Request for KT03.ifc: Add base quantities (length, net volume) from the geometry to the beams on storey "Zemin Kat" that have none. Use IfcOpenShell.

First a look at what the model holds.

```python
import ifcopenshell
import ifcopenshell.util.element
import ifcopenshell.util.unit

model = ifcopenshell.open("KT03.ifc")
print(model.schema)
for unit_type in ("LENGTHUNIT", "AREAUNIT", "VOLUMEUNIT"):
    print(unit_type, ifcopenshell.util.unit.calculate_unit_scale(model, unit_type))
storey = next(s for s in model.by_type("IfcBuildingStorey") if s.Name == "Zemin Kat")
beams = [e for e in ifcopenshell.util.element.get_decomposition(storey) if e.is_a("IfcBeam")]
for e in sorted(beams, key=lambda e: e.id()):
    print(e.id(), e.is_a(), e.Name, list(ifcopenshell.util.element.get_psets(e, qtos_only=True)), sep=" | ")
```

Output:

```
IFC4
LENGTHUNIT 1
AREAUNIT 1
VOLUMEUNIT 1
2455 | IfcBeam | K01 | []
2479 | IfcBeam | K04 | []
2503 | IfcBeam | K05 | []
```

```python
import ifcopenshell
import ifcopenshell.api.pset
import ifcopenshell.geom
import ifcopenshell.util.element
import ifcopenshell.util.shape
import ifcopenshell.util.unit

model = ifcopenshell.open("KT03.ifc")
unit_scale = ifcopenshell.util.unit.calculate_unit_scale(model)
volume_scale = ifcopenshell.util.unit.calculate_unit_scale(model, "VOLUMEUNIT")
settings = ifcopenshell.geom.settings()

storey = next(s for s in model.by_type("IfcBuildingStorey") if s.Name == "Zemin Kat")
beams = [e for e in ifcopenshell.util.element.get_decomposition(storey) if e.is_a("IfcBeam")]

for e in sorted(beams, key=lambda e: e.id()):
    if ifcopenshell.util.element.get_psets(e, qtos_only=True, should_inherit=False):
        continue
    # Geometry comes back in metres, in the element's own axes.
    shape = ifcopenshell.geom.create_shape(settings, e)
    values = {
        "Length": ifcopenshell.util.shape.get_max_xyz(shape.geometry) / unit_scale,
        "NetVolume": ifcopenshell.util.shape.get_volume(shape.geometry) / volume_scale,
    }
    qto = ifcopenshell.api.pset.add_qto(model, product=e, name="Qto_BeamBaseQuantities")
    ifcopenshell.api.pset.edit_qto(model, qto=qto, properties=values)
    print(e.id(), {k: round(v, 3) for k, v in values.items()})

model.write("KT03_updated.ifc")
```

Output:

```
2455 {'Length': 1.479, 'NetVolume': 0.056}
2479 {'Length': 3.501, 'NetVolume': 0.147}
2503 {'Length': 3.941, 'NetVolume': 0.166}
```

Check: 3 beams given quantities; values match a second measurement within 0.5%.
